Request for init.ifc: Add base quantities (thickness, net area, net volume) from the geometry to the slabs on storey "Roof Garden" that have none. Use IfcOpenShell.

First a look at what the model holds.

```python
import ifcopenshell
import ifcopenshell.util.element
import ifcopenshell.util.unit

model = ifcopenshell.open("init.ifc")
print(model.schema)
for unit_type in ("LENGTHUNIT", "AREAUNIT", "VOLUMEUNIT"):
    print(unit_type, ifcopenshell.util.unit.calculate_unit_scale(model, unit_type))
storey = next(s for s in model.by_type("IfcBuildingStorey") if s.Name == "Roof Garden")
slabs = [e for e in ifcopenshell.util.element.get_decomposition(storey) if e.is_a("IfcSlab")]
for e in sorted(slabs, key=lambda e: e.id()):
    print(e.id(), e.is_a(), e.Name, list(ifcopenshell.util.element.get_psets(e, qtos_only=True)), sep=" | ")
```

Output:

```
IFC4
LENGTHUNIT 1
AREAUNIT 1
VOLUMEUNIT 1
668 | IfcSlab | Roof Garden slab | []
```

```python
import ifcopenshell
import ifcopenshell.api.pset
import ifcopenshell.geom
import ifcopenshell.util.element
import ifcopenshell.util.shape
import ifcopenshell.util.unit

model = ifcopenshell.open("init.ifc")
unit_scale = ifcopenshell.util.unit.calculate_unit_scale(model)
area_scale = ifcopenshell.util.unit.calculate_unit_scale(model, "AREAUNIT")
volume_scale = ifcopenshell.util.unit.calculate_unit_scale(model, "VOLUMEUNIT")
settings = ifcopenshell.geom.settings()

storey = next(s for s in model.by_type("IfcBuildingStorey") if s.Name == "Roof Garden")
slabs = [e for e in ifcopenshell.util.element.get_decomposition(storey) if e.is_a("IfcSlab")]

for e in sorted(slabs, key=lambda e: e.id()):
    if ifcopenshell.util.element.get_psets(e, qtos_only=True, should_inherit=False):
        continue
    # Geometry comes back in metres, in the element's own axes.
    shape = ifcopenshell.geom.create_shape(settings, e)
    values = {
        "Width": ifcopenshell.util.shape.get_z(shape.geometry) / unit_scale,
        "NetArea": ifcopenshell.util.shape.get_footprint_area(shape.geometry) / area_scale,
        "NetVolume": ifcopenshell.util.shape.get_volume(shape.geometry) / volume_scale,
    }
    qto = ifcopenshell.api.pset.add_qto(model, product=e, name="Qto_SlabBaseQuantities")
    ifcopenshell.api.pset.edit_qto(model, qto=qto, properties=values)
    print(e.id(), {k: round(v, 3) for k, v in values.items()})

model.write("init-out.ifc")
```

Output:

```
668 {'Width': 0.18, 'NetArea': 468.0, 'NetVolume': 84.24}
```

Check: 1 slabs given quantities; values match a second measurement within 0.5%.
